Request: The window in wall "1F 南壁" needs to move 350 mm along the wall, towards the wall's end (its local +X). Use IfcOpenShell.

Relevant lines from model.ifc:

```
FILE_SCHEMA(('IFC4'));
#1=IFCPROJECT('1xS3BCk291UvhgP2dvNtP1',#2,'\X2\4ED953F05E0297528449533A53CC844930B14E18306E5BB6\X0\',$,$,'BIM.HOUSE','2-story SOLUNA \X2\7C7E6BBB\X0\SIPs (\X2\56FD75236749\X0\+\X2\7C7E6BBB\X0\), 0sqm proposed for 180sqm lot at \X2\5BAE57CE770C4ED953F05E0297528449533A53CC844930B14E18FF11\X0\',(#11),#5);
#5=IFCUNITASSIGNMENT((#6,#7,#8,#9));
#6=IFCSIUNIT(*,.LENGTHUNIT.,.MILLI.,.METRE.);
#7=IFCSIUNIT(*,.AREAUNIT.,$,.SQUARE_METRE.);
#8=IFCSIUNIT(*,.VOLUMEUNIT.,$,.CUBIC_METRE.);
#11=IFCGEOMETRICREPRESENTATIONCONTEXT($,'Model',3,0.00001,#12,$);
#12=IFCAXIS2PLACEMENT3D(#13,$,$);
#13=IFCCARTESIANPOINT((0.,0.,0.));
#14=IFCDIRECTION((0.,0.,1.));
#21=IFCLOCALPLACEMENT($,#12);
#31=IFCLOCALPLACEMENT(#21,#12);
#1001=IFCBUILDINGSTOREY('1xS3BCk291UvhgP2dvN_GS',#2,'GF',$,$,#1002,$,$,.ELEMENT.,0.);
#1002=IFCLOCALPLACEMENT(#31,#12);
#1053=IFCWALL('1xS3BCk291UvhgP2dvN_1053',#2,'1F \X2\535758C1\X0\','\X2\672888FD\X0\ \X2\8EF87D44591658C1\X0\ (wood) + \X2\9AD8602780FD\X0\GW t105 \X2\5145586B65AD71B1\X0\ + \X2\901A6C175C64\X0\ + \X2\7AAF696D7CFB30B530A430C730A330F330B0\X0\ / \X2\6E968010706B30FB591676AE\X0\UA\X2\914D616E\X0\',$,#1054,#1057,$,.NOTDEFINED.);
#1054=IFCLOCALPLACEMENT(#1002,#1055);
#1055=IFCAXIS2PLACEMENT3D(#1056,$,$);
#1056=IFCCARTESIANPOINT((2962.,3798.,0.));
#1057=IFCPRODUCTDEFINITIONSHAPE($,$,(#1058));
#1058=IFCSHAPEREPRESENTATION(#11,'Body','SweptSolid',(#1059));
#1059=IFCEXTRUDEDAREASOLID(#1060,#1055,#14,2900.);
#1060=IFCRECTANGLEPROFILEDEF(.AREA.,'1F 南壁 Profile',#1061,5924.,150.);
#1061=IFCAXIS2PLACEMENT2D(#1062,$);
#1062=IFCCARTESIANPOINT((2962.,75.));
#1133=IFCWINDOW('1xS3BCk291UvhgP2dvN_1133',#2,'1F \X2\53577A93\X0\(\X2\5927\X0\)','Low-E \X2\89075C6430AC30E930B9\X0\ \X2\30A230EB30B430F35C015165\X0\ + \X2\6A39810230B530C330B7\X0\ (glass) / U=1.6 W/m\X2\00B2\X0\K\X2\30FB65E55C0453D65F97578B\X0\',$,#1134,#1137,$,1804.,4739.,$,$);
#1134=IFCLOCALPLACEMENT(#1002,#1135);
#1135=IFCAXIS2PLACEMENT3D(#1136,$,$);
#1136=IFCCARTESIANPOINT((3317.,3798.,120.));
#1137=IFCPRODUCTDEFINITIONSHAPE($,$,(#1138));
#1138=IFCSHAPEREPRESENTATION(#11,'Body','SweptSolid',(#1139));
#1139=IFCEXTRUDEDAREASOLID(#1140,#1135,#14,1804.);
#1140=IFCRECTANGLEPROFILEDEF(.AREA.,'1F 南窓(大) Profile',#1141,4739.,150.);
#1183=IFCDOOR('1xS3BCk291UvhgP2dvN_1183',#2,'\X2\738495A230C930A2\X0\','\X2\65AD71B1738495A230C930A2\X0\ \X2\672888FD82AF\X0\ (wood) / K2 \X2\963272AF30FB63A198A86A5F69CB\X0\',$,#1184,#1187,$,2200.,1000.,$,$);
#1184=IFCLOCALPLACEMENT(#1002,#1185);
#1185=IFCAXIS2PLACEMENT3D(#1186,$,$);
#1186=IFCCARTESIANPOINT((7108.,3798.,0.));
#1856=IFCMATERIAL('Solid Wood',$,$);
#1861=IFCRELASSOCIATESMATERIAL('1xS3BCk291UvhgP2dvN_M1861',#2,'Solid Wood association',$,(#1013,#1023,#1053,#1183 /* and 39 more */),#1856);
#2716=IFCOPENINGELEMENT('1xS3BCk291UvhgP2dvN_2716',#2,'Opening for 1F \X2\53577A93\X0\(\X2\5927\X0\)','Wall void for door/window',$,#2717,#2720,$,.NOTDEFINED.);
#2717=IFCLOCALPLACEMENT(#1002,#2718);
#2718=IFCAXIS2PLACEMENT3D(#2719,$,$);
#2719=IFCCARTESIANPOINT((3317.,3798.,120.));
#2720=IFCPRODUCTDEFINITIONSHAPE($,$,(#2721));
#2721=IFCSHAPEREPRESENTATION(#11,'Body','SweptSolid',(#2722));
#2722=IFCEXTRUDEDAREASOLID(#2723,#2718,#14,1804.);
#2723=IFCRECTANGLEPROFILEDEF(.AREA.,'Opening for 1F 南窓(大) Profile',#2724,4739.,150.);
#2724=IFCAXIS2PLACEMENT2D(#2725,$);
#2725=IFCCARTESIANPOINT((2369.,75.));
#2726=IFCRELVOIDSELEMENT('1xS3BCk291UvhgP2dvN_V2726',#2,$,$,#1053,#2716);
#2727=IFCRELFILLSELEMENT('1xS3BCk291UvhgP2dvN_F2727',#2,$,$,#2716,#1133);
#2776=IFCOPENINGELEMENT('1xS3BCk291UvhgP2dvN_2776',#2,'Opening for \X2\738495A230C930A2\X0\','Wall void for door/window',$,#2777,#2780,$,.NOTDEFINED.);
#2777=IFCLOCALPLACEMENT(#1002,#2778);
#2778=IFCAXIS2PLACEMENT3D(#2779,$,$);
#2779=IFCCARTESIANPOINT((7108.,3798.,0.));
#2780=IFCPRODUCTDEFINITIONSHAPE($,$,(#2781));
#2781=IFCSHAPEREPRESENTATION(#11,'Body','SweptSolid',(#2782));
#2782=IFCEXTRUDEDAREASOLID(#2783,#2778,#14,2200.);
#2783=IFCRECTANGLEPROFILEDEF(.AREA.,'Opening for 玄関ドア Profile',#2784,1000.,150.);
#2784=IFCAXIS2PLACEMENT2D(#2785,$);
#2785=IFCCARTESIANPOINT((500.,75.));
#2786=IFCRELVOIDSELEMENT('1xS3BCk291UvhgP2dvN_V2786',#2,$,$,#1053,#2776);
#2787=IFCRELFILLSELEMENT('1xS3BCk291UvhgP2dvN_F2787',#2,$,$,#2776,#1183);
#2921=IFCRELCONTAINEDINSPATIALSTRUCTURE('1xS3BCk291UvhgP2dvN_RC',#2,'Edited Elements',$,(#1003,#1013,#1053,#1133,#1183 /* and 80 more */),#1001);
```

```python
import ifcopenshell
import ifcopenshell.api.geometry
import ifcopenshell.util.placement
import ifcopenshell.util.unit

model = ifcopenshell.open("model.ifc")
unit_scale = ifcopenshell.util.unit.calculate_unit_scale(model)

window = model.by_guid("1xS3BCk291UvhgP2dvN_1133")
opening = window.FillsVoids[0].RelatingOpeningElement
wall = opening.VoidsElements[0].RelatingBuildingElement

wall_matrix = ifcopenshell.util.placement.get_local_placement(wall.ObjectPlacement)
shift = wall_matrix[:3, 0] * 0.35 / unit_scale
before = ifcopenshell.util.placement.get_local_placement(window.ObjectPlacement)[:3, 3].copy()

# The window is not placed relative to its opening, so move both.
for product in (opening, window):
    matrix = ifcopenshell.util.placement.get_local_placement(product.ObjectPlacement)
    matrix[:3, 3] += shift
    ifcopenshell.api.geometry.edit_object_placement(model, product=product, matrix=matrix, is_si=False)

after = ifcopenshell.util.placement.get_local_placement(window.ObjectPlacement)[:3, 3]
print("window moved by", (after - before).round(3) + 0.0)

model.write("model_edited.ifc")
```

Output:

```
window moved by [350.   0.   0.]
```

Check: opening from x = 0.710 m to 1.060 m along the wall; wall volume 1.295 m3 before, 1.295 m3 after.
